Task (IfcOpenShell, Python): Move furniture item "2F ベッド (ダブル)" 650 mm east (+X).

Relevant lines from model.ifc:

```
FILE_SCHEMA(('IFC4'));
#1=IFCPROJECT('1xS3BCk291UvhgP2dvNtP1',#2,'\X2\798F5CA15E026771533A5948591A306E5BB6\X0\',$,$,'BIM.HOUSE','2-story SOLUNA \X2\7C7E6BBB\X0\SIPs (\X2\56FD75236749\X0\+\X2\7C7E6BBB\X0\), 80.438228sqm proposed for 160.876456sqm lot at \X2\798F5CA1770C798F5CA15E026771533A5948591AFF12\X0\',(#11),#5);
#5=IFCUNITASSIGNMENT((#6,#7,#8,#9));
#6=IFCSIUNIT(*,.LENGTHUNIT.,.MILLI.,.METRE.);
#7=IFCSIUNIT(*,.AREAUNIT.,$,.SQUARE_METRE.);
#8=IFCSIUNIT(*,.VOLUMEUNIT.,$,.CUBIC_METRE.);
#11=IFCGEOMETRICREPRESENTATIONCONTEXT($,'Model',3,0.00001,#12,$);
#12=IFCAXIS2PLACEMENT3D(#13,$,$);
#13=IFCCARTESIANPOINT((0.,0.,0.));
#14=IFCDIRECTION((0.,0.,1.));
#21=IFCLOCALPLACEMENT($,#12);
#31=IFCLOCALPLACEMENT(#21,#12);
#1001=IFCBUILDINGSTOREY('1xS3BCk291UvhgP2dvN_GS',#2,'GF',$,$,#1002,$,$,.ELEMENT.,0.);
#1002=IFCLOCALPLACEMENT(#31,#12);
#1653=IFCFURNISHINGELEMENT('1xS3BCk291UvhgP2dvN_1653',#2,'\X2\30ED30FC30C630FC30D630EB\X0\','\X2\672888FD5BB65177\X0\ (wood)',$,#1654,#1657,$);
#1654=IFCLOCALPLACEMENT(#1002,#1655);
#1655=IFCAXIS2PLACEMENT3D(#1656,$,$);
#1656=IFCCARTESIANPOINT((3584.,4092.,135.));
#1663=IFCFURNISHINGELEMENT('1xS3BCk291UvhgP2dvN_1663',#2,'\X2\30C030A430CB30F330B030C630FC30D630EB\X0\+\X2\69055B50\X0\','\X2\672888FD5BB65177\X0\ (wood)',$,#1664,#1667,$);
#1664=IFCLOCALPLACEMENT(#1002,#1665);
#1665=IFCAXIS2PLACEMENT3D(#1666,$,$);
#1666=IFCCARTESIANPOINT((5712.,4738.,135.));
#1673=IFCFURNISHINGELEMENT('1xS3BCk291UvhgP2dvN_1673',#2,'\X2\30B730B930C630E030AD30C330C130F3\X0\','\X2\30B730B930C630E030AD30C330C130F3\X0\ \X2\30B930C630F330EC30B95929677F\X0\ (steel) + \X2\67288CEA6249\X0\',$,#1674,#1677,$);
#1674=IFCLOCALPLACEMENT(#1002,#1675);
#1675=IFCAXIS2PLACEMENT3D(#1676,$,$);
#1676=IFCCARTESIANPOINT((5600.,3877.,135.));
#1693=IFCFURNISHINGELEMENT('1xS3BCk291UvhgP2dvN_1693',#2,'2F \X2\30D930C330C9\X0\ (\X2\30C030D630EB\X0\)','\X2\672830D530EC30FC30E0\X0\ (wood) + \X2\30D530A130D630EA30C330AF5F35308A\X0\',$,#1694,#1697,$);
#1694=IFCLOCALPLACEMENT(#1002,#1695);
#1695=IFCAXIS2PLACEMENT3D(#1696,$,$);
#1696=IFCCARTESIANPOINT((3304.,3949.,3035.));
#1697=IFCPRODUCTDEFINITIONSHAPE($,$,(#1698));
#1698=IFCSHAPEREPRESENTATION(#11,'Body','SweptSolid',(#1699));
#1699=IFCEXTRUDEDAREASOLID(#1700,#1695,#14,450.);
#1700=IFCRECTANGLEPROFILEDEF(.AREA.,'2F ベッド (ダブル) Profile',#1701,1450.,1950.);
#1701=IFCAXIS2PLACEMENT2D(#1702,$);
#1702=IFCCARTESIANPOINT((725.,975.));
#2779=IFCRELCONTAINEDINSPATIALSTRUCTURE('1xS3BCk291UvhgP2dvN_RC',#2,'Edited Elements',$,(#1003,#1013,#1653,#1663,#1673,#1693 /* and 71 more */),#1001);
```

```python
import ifcopenshell
import ifcopenshell.api.geometry
import ifcopenshell.util.placement
import ifcopenshell.util.unit

model = ifcopenshell.open("model.ifc")
unit_scale = ifcopenshell.util.unit.calculate_unit_scale(model)

item = model.by_guid("1xS3BCk291UvhgP2dvN_1693")
matrix = ifcopenshell.util.placement.get_local_placement(item.ObjectPlacement)
matrix[0, 3] += 0.65 / unit_scale
ifcopenshell.api.geometry.edit_object_placement(model, product=item, matrix=matrix, is_si=False)

print(ifcopenshell.util.placement.get_local_placement(item.ObjectPlacement).round(3) + 0.0)

model.write("model_edited.ifc")
```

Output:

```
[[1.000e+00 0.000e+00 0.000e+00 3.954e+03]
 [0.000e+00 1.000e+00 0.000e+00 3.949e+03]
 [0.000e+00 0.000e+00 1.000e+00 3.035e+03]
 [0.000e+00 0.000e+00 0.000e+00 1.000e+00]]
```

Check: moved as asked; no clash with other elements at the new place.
